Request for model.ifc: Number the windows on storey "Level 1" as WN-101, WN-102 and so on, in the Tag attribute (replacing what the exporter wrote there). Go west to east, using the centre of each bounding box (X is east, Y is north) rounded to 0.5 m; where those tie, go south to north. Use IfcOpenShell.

First a look at what the model holds.

```python
import ifcopenshell
import ifcopenshell.util.element
import ifcopenshell.util.placement

model = ifcopenshell.open("model.ifc")
print(model.schema)
storey = next(s for s in model.by_type("IfcBuildingStorey") if s.Name == "Level 1")
windows = [e for e in ifcopenshell.util.element.get_decomposition(storey) if e.is_a("IfcWindow")]
for e in sorted(windows, key=lambda e: e.id()):
    origin = ifcopenshell.util.placement.get_local_placement(e.ObjectPlacement)[:3, 3]
    print(e.id(), e.Tag, e.Name, origin.round(2) + 0.0, sep=" | ")
```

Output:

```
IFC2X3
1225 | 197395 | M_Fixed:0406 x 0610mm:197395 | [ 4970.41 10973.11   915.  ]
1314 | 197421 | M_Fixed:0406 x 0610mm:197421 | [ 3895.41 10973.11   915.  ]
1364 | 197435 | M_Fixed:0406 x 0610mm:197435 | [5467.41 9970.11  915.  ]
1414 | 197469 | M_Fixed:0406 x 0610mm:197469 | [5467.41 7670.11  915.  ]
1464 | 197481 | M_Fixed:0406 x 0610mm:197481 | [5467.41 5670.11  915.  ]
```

```python
import ifcopenshell
import ifcopenshell.geom
import ifcopenshell.util.element
import ifcopenshell.util.shape

model = ifcopenshell.open("model.ifc")
settings = ifcopenshell.geom.settings()
settings.set("use-world-coords", True)


def centre(element):
    shape = ifcopenshell.geom.create_shape(settings, element)
    return ifcopenshell.util.shape.get_bbox_centroid(shape.geometry)


storey = next(s for s in model.by_type("IfcBuildingStorey") if s.Name == "Level 1")
windows = [e for e in ifcopenshell.util.element.get_decomposition(storey) if e.is_a("IfcWindow")]

# Insertion points can sit at a corner or the storey origin, so sort by the geometry (in metres).
centres = {e: centre(e) for e in windows}
windows.sort(key=lambda e: (round(centres[e][0] / 0.5), centres[e][1]))

for i, e in enumerate(windows, start=1):
    number = f"WN-1{i:02d}"
    e.Tag = number
    print(e.id(), number)

model.write("model-out.ifc")
```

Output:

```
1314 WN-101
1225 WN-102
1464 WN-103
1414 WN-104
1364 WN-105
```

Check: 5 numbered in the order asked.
